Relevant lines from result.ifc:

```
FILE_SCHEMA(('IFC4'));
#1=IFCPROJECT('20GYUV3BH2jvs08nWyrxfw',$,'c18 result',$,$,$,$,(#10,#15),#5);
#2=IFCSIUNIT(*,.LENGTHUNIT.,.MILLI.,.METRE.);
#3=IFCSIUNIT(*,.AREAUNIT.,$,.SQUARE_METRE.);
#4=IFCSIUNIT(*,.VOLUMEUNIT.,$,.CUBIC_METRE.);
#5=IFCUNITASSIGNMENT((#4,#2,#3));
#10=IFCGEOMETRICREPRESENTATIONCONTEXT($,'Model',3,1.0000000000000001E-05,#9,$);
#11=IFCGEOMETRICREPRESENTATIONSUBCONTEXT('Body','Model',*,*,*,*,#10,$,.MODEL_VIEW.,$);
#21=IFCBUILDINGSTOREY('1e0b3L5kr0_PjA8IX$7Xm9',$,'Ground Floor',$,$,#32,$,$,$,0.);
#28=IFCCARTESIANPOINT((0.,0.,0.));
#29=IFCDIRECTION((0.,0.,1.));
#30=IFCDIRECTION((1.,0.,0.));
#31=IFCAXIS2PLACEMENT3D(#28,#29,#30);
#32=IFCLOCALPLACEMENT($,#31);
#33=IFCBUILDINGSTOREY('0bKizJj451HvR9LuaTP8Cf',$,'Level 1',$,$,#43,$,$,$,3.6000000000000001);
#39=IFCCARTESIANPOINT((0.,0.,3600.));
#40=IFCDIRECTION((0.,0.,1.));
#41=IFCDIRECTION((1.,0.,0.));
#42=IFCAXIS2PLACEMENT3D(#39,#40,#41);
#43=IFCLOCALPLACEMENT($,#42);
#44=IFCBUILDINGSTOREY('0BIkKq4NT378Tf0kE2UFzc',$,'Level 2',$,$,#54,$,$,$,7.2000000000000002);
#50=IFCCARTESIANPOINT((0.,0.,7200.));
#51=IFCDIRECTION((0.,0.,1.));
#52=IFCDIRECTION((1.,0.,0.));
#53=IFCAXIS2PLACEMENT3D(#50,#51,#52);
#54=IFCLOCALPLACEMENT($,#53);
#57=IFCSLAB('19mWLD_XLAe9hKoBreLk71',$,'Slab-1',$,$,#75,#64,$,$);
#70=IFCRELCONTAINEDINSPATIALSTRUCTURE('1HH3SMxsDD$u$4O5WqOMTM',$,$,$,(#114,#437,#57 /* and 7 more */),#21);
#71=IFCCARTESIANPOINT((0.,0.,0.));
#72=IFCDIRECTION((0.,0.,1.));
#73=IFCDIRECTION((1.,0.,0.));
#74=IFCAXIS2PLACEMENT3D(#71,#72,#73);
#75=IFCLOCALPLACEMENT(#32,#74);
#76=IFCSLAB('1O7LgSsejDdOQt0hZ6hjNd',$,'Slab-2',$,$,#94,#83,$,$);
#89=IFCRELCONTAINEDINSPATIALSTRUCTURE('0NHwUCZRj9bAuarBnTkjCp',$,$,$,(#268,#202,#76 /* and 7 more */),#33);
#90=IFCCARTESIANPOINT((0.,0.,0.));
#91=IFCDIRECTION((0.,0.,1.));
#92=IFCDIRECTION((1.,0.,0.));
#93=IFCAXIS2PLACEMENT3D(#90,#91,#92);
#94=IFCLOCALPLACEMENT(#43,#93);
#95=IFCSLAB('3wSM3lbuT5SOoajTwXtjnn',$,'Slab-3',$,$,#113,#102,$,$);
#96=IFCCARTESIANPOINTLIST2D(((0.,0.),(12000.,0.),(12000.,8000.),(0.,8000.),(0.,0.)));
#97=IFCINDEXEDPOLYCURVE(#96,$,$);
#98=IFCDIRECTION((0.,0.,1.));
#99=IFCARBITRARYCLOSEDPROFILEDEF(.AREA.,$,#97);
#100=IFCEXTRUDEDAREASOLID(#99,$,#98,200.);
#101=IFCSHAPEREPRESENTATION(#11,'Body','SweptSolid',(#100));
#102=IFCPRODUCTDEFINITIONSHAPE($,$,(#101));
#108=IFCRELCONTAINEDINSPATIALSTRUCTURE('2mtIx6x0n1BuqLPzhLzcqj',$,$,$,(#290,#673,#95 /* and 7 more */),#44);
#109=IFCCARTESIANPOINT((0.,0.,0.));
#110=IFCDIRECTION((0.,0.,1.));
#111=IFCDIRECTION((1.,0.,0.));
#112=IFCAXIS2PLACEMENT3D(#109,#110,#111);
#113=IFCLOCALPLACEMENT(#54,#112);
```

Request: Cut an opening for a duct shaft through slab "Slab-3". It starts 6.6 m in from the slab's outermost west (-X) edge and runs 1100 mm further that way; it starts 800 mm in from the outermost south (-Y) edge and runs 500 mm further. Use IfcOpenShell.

```python
import numpy as np
import ifcopenshell
import ifcopenshell.api.feature
import ifcopenshell.api.geometry
import ifcopenshell.api.root
import ifcopenshell.geom
import ifcopenshell.util.placement
import ifcopenshell.util.representation
import ifcopenshell.util.shape
import ifcopenshell.util.unit

model = ifcopenshell.open("result.ifc")
unit_scale = ifcopenshell.util.unit.calculate_unit_scale(model)
settings = ifcopenshell.geom.settings()


def volume(element):
    """Net volume in cubic metres, openings subtracted."""
    shape = ifcopenshell.geom.create_shape(settings, element)
    return ifcopenshell.util.shape.get_volume(shape.geometry)


slab = model.by_guid("3wSM3lbuT5SOoajTwXtjnn")
before = volume(slab)

# Extent in the slab's own axes, in metres. The edges named are its -X and -Y sides.
slab_shape = ifcopenshell.geom.create_shape(settings, slab)
vertices = ifcopenshell.util.shape.get_vertices(slab_shape.geometry)
x_min, y_min, bottom = vertices.min(axis=0)
top = vertices[:, 2].max()

opening = ifcopenshell.api.root.create_entity(model, ifc_class="IfcOpeningElement", name="Duct shaft opening", predefined_type="OPENING")
context = ifcopenshell.util.representation.get_context(model, "Model", "Body", "MODEL_VIEW")
width, depth = 1.1, 0.5
outline = [(0.0, 0.0), (width, 0.0), (width, depth), (0.0, depth), (0.0, 0.0)]
# Overshoot both faces by 50 mm so the cut is clean.
shape = ifcopenshell.api.geometry.add_slab_representation(
    model, context=context, depth=top - bottom + 0.1, polyline=outline
)
ifcopenshell.api.geometry.assign_representation(model, product=opening, representation=shape)

matrix = ifcopenshell.util.placement.get_local_placement(slab.ObjectPlacement)
matrix[:, 3] = matrix @ np.append(np.array([x_min + 6.6, y_min + 0.8, bottom - 0.05]) / unit_scale, 1.0)
ifcopenshell.api.geometry.edit_object_placement(model, product=opening, matrix=matrix, is_si=False)
ifcopenshell.api.feature.add_feature(model, feature=opening, element=slab)

after = volume(slab)

print(f"slab volume {before:.3f} -> {after:.3f} m3")

model.write("result-out.ifc")
```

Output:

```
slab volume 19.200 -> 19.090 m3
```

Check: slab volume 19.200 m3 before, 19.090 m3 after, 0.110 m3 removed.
